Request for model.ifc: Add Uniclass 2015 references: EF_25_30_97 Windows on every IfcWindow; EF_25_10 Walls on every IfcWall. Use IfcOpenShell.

First a look at what the model holds.

```python
import ifcopenshell

model = ifcopenshell.open("model.ifc")
print(model.schema)
print("classifications:", [c.Name for c in model.by_type("IfcClassification")])
for ifc_class in ("IfcDoor", "IfcRoof", "IfcStair", "IfcWall", "IfcWindow"):
    print(ifc_class, len(model.by_type(ifc_class)))
```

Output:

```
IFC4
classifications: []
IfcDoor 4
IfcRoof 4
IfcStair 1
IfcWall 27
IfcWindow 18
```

```python
import ifcopenshell
import ifcopenshell.api.classification

model = ifcopenshell.open("model.ifc")

system = ifcopenshell.api.classification.add_classification(model, classification="Uniclass 2015")

codes = {
    "IfcWindow": ("EF_25_30_97", "Windows"),
    "IfcWall": ("EF_25_10", "Walls"),
}
for ifc_class, (code, name) in codes.items():
    products = model.by_type(ifc_class)
    ifcopenshell.api.classification.add_reference(
        model, products=products, classification=system, identification=code, name=name
    )
    print(code, len(products))

model.write("model-out.ifc")
```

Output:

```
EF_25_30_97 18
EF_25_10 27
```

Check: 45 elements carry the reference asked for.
